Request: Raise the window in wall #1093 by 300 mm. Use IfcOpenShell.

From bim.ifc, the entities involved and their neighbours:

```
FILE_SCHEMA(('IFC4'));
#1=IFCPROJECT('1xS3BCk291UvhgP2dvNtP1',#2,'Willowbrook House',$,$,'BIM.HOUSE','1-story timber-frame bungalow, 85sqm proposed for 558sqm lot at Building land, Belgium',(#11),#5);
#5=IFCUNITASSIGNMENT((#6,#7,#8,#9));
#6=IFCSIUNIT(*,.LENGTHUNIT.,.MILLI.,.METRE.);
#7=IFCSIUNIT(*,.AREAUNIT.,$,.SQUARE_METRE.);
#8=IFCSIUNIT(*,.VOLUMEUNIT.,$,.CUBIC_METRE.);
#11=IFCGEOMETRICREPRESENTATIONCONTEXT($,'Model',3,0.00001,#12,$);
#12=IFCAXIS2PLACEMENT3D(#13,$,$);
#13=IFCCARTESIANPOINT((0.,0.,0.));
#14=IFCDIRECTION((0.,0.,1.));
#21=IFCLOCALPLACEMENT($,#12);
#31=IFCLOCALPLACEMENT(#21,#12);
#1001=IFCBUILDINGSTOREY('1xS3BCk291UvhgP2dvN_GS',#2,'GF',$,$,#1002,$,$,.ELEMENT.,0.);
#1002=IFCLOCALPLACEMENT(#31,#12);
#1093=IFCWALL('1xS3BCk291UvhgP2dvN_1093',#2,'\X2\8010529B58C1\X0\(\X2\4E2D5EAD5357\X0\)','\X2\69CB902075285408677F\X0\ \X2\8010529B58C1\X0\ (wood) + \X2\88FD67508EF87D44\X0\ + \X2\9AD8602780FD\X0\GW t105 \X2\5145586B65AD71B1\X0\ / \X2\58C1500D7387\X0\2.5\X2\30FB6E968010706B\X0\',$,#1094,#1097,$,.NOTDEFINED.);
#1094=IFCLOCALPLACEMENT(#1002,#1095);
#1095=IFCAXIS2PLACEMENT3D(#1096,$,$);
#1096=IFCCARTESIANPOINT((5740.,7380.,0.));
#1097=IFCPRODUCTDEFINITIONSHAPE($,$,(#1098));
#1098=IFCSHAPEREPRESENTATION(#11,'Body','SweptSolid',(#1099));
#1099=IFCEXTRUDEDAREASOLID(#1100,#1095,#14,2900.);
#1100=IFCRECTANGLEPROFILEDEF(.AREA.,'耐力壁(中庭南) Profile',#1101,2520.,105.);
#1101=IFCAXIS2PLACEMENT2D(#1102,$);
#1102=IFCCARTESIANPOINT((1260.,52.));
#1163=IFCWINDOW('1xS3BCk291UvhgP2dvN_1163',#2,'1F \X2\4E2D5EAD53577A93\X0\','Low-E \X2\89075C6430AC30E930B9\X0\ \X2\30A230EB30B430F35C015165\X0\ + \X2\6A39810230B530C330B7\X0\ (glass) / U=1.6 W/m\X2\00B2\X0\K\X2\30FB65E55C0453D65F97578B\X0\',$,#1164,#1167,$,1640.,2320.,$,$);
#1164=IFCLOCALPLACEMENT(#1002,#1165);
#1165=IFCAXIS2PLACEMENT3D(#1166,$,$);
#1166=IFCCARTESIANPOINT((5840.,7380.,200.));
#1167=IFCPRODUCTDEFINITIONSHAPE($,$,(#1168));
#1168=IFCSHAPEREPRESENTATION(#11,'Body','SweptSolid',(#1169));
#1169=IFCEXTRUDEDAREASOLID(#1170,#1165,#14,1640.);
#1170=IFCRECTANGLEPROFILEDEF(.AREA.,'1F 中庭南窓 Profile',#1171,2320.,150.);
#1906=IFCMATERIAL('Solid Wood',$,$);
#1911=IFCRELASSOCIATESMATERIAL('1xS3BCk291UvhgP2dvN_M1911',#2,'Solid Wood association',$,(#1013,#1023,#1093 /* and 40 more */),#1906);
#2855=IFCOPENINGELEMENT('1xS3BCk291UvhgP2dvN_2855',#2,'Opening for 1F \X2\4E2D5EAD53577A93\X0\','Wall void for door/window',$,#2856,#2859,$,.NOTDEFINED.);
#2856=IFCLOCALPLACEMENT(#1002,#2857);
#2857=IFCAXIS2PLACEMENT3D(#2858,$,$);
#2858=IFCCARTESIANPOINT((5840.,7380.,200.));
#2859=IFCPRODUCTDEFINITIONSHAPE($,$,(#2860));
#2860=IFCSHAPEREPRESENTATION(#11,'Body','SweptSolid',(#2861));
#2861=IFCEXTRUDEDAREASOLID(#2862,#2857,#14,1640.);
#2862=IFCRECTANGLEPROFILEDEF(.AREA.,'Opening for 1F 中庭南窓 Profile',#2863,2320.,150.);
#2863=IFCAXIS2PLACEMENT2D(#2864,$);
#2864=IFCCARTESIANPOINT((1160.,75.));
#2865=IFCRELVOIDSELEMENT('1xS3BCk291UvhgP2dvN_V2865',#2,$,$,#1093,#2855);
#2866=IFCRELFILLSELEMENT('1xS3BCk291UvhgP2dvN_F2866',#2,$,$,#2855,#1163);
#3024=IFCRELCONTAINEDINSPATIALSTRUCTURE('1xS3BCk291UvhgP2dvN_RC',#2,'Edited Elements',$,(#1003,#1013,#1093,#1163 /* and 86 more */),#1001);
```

```python
import numpy as np
import ifcopenshell
import ifcopenshell.api.geometry
import ifcopenshell.util.placement
import ifcopenshell.util.unit

model = ifcopenshell.open("bim.ifc")
unit_scale = ifcopenshell.util.unit.calculate_unit_scale(model)

window = model.by_guid("1xS3BCk291UvhgP2dvN_1163")
opening = window.FillsVoids[0].RelatingOpeningElement
dz = 0.3 / unit_scale

shift = np.array([0.0, 0.0, dz])
# The window is not placed relative to its opening, so move both.
for product in (opening, window):
    matrix = ifcopenshell.util.placement.get_local_placement(product.ObjectPlacement)
    matrix[:3, 3] += shift
    ifcopenshell.api.geometry.edit_object_placement(model, product=product, matrix=matrix, is_si=False)

print(f"moved by {dz * unit_scale:+.3f} m")

model.write("bim_updated.ifc")
```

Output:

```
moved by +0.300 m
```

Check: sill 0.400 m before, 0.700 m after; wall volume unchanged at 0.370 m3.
